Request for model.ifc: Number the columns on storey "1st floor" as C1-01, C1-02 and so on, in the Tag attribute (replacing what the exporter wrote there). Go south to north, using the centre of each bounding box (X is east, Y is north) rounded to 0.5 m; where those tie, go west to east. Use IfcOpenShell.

First a look at what the model holds.

```python
import ifcopenshell
import ifcopenshell.util.element
import ifcopenshell.util.placement

model = ifcopenshell.open("model.ifc")
print(model.schema)
storey = next(s for s in model.by_type("IfcBuildingStorey") if s.Name == "1st floor")
columns = [e for e in ifcopenshell.util.element.get_decomposition(storey) if e.is_a("IfcColumn")]
for e in sorted(columns, key=lambda e: e.id()):
    origin = ifcopenshell.util.placement.get_local_placement(e.ObjectPlacement)[:3, 3]
    print(e.id(), e.Tag, e.Name, origin.round(2) + 0.0, sep=" | ")
```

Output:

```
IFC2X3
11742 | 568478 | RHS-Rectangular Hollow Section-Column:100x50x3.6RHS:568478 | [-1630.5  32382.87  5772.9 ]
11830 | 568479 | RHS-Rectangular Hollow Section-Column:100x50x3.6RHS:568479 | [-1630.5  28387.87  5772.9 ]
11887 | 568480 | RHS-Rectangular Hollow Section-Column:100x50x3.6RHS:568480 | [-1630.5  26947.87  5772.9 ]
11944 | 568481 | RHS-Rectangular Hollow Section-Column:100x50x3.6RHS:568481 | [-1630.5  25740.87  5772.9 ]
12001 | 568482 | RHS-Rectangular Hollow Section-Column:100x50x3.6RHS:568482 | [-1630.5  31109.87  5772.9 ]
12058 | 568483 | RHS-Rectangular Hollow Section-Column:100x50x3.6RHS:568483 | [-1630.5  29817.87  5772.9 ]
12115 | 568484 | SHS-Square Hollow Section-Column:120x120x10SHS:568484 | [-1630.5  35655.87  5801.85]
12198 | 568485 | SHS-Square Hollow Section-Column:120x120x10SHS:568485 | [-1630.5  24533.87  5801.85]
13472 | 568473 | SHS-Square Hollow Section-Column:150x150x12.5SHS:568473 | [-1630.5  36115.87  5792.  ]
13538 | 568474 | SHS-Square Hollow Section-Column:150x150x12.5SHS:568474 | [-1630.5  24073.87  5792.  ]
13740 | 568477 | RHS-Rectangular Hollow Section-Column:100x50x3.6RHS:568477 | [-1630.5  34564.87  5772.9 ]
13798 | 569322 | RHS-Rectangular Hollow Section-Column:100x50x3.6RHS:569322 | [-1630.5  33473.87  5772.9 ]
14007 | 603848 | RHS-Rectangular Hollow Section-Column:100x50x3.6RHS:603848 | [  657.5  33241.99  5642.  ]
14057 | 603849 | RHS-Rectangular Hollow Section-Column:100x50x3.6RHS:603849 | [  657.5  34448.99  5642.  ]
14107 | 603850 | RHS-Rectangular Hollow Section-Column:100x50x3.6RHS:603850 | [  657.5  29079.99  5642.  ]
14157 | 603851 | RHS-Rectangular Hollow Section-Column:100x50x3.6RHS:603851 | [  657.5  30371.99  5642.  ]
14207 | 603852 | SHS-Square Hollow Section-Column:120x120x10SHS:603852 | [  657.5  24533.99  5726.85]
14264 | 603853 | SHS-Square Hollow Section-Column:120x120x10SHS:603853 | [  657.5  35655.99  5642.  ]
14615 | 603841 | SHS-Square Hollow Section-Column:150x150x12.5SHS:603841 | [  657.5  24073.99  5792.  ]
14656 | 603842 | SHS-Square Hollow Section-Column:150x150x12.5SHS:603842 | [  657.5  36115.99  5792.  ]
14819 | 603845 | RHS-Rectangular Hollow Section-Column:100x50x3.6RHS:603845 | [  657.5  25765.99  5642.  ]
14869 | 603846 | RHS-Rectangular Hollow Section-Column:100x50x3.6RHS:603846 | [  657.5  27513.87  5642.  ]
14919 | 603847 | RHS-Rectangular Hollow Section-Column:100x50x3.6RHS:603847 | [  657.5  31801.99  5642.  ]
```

```python
import ifcopenshell
import ifcopenshell.geom
import ifcopenshell.util.element
import ifcopenshell.util.shape

model = ifcopenshell.open("model.ifc")
settings = ifcopenshell.geom.settings()
settings.set("use-world-coords", True)


def centre(element):
    shape = ifcopenshell.geom.create_shape(settings, element)
    return ifcopenshell.util.shape.get_bbox_centroid(shape.geometry)


storey = next(s for s in model.by_type("IfcBuildingStorey") if s.Name == "1st floor")
columns = [e for e in ifcopenshell.util.element.get_decomposition(storey) if e.is_a("IfcColumn")]

# Insertion points can sit at a corner or the storey origin, so sort by the geometry (in metres).
centres = {e: centre(e) for e in columns}
columns.sort(key=lambda e: (round(centres[e][1] / 0.5), centres[e][0]))

for i, e in enumerate(columns, start=1):
    number = f"C1-{i:02d}"
    e.Tag = number
    print(e.id(), number)

model.write("model_v2.ifc")
```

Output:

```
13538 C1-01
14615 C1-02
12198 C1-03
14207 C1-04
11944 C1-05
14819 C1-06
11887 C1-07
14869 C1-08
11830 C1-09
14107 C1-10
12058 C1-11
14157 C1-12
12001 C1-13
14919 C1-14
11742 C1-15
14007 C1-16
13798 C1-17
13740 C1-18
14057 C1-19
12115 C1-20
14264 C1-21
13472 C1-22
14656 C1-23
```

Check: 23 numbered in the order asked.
